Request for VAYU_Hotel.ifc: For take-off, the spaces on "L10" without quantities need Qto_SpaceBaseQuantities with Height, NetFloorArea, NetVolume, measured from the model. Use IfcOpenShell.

First a look at what the model holds.

```python
import ifcopenshell
import ifcopenshell.util.element
import ifcopenshell.util.unit

model = ifcopenshell.open("VAYU_Hotel.ifc")
print(model.schema)
for unit_type in ("LENGTHUNIT", "AREAUNIT", "VOLUMEUNIT"):
    print(unit_type, ifcopenshell.util.unit.calculate_unit_scale(model, unit_type))
storey = next(s for s in model.by_type("IfcBuildingStorey") if s.Name == "L10")
spaces = [e for e in ifcopenshell.util.element.get_decomposition(storey) if e.is_a("IfcSpace")]
for e in sorted(spaces, key=lambda e: e.id()):
    print(e.id(), e.is_a(), e.Name, list(ifcopenshell.util.element.get_psets(e, qtos_only=True)), sep=" | ")
```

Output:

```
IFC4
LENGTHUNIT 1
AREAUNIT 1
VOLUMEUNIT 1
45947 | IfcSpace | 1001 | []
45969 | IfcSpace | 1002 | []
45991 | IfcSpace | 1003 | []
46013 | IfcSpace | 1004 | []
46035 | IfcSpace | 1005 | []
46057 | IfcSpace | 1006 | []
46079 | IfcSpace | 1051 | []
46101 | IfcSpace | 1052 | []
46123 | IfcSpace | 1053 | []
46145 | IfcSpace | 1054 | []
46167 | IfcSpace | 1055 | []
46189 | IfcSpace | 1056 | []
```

```python
import ifcopenshell
import ifcopenshell.api.pset
import ifcopenshell.geom
import ifcopenshell.util.element
import ifcopenshell.util.shape
import ifcopenshell.util.unit

model = ifcopenshell.open("VAYU_Hotel.ifc")
unit_scale = ifcopenshell.util.unit.calculate_unit_scale(model)
area_scale = ifcopenshell.util.unit.calculate_unit_scale(model, "AREAUNIT")
volume_scale = ifcopenshell.util.unit.calculate_unit_scale(model, "VOLUMEUNIT")
settings = ifcopenshell.geom.settings()

storey = next(s for s in model.by_type("IfcBuildingStorey") if s.Name == "L10")
spaces = [e for e in ifcopenshell.util.element.get_decomposition(storey) if e.is_a("IfcSpace")]

for e in sorted(spaces, key=lambda e: e.id()):
    if ifcopenshell.util.element.get_psets(e, qtos_only=True, should_inherit=False):
        continue
    # Geometry comes back in metres, in the element's own axes.
    shape = ifcopenshell.geom.create_shape(settings, e)
    values = {
        "Height": ifcopenshell.util.shape.get_z(shape.geometry) / unit_scale,
        "NetFloorArea": ifcopenshell.util.shape.get_footprint_area(shape.geometry) / area_scale,
        "NetVolume": ifcopenshell.util.shape.get_volume(shape.geometry) / volume_scale,
    }
    qto = ifcopenshell.api.pset.add_qto(model, product=e, name="Qto_SpaceBaseQuantities")
    ifcopenshell.api.pset.edit_qto(model, qto=qto, properties=values)
    print(e.id(), {k: round(v, 3) for k, v in values.items()})

model.write("VAYU_Hotel_rev.ifc")
```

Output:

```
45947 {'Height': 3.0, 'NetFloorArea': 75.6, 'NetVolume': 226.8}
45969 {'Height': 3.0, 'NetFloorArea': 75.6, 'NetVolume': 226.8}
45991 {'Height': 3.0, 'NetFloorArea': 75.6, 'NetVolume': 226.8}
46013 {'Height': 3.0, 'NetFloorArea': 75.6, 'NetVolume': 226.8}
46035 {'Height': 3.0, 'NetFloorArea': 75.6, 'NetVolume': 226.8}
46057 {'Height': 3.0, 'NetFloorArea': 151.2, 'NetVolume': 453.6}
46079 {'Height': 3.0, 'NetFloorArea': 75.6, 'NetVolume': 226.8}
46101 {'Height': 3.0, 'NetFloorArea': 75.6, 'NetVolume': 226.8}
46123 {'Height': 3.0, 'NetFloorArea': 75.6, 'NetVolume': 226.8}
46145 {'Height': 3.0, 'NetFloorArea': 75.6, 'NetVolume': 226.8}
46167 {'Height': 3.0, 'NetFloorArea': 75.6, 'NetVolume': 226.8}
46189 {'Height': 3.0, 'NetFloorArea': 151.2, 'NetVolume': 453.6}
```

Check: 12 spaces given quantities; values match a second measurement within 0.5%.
